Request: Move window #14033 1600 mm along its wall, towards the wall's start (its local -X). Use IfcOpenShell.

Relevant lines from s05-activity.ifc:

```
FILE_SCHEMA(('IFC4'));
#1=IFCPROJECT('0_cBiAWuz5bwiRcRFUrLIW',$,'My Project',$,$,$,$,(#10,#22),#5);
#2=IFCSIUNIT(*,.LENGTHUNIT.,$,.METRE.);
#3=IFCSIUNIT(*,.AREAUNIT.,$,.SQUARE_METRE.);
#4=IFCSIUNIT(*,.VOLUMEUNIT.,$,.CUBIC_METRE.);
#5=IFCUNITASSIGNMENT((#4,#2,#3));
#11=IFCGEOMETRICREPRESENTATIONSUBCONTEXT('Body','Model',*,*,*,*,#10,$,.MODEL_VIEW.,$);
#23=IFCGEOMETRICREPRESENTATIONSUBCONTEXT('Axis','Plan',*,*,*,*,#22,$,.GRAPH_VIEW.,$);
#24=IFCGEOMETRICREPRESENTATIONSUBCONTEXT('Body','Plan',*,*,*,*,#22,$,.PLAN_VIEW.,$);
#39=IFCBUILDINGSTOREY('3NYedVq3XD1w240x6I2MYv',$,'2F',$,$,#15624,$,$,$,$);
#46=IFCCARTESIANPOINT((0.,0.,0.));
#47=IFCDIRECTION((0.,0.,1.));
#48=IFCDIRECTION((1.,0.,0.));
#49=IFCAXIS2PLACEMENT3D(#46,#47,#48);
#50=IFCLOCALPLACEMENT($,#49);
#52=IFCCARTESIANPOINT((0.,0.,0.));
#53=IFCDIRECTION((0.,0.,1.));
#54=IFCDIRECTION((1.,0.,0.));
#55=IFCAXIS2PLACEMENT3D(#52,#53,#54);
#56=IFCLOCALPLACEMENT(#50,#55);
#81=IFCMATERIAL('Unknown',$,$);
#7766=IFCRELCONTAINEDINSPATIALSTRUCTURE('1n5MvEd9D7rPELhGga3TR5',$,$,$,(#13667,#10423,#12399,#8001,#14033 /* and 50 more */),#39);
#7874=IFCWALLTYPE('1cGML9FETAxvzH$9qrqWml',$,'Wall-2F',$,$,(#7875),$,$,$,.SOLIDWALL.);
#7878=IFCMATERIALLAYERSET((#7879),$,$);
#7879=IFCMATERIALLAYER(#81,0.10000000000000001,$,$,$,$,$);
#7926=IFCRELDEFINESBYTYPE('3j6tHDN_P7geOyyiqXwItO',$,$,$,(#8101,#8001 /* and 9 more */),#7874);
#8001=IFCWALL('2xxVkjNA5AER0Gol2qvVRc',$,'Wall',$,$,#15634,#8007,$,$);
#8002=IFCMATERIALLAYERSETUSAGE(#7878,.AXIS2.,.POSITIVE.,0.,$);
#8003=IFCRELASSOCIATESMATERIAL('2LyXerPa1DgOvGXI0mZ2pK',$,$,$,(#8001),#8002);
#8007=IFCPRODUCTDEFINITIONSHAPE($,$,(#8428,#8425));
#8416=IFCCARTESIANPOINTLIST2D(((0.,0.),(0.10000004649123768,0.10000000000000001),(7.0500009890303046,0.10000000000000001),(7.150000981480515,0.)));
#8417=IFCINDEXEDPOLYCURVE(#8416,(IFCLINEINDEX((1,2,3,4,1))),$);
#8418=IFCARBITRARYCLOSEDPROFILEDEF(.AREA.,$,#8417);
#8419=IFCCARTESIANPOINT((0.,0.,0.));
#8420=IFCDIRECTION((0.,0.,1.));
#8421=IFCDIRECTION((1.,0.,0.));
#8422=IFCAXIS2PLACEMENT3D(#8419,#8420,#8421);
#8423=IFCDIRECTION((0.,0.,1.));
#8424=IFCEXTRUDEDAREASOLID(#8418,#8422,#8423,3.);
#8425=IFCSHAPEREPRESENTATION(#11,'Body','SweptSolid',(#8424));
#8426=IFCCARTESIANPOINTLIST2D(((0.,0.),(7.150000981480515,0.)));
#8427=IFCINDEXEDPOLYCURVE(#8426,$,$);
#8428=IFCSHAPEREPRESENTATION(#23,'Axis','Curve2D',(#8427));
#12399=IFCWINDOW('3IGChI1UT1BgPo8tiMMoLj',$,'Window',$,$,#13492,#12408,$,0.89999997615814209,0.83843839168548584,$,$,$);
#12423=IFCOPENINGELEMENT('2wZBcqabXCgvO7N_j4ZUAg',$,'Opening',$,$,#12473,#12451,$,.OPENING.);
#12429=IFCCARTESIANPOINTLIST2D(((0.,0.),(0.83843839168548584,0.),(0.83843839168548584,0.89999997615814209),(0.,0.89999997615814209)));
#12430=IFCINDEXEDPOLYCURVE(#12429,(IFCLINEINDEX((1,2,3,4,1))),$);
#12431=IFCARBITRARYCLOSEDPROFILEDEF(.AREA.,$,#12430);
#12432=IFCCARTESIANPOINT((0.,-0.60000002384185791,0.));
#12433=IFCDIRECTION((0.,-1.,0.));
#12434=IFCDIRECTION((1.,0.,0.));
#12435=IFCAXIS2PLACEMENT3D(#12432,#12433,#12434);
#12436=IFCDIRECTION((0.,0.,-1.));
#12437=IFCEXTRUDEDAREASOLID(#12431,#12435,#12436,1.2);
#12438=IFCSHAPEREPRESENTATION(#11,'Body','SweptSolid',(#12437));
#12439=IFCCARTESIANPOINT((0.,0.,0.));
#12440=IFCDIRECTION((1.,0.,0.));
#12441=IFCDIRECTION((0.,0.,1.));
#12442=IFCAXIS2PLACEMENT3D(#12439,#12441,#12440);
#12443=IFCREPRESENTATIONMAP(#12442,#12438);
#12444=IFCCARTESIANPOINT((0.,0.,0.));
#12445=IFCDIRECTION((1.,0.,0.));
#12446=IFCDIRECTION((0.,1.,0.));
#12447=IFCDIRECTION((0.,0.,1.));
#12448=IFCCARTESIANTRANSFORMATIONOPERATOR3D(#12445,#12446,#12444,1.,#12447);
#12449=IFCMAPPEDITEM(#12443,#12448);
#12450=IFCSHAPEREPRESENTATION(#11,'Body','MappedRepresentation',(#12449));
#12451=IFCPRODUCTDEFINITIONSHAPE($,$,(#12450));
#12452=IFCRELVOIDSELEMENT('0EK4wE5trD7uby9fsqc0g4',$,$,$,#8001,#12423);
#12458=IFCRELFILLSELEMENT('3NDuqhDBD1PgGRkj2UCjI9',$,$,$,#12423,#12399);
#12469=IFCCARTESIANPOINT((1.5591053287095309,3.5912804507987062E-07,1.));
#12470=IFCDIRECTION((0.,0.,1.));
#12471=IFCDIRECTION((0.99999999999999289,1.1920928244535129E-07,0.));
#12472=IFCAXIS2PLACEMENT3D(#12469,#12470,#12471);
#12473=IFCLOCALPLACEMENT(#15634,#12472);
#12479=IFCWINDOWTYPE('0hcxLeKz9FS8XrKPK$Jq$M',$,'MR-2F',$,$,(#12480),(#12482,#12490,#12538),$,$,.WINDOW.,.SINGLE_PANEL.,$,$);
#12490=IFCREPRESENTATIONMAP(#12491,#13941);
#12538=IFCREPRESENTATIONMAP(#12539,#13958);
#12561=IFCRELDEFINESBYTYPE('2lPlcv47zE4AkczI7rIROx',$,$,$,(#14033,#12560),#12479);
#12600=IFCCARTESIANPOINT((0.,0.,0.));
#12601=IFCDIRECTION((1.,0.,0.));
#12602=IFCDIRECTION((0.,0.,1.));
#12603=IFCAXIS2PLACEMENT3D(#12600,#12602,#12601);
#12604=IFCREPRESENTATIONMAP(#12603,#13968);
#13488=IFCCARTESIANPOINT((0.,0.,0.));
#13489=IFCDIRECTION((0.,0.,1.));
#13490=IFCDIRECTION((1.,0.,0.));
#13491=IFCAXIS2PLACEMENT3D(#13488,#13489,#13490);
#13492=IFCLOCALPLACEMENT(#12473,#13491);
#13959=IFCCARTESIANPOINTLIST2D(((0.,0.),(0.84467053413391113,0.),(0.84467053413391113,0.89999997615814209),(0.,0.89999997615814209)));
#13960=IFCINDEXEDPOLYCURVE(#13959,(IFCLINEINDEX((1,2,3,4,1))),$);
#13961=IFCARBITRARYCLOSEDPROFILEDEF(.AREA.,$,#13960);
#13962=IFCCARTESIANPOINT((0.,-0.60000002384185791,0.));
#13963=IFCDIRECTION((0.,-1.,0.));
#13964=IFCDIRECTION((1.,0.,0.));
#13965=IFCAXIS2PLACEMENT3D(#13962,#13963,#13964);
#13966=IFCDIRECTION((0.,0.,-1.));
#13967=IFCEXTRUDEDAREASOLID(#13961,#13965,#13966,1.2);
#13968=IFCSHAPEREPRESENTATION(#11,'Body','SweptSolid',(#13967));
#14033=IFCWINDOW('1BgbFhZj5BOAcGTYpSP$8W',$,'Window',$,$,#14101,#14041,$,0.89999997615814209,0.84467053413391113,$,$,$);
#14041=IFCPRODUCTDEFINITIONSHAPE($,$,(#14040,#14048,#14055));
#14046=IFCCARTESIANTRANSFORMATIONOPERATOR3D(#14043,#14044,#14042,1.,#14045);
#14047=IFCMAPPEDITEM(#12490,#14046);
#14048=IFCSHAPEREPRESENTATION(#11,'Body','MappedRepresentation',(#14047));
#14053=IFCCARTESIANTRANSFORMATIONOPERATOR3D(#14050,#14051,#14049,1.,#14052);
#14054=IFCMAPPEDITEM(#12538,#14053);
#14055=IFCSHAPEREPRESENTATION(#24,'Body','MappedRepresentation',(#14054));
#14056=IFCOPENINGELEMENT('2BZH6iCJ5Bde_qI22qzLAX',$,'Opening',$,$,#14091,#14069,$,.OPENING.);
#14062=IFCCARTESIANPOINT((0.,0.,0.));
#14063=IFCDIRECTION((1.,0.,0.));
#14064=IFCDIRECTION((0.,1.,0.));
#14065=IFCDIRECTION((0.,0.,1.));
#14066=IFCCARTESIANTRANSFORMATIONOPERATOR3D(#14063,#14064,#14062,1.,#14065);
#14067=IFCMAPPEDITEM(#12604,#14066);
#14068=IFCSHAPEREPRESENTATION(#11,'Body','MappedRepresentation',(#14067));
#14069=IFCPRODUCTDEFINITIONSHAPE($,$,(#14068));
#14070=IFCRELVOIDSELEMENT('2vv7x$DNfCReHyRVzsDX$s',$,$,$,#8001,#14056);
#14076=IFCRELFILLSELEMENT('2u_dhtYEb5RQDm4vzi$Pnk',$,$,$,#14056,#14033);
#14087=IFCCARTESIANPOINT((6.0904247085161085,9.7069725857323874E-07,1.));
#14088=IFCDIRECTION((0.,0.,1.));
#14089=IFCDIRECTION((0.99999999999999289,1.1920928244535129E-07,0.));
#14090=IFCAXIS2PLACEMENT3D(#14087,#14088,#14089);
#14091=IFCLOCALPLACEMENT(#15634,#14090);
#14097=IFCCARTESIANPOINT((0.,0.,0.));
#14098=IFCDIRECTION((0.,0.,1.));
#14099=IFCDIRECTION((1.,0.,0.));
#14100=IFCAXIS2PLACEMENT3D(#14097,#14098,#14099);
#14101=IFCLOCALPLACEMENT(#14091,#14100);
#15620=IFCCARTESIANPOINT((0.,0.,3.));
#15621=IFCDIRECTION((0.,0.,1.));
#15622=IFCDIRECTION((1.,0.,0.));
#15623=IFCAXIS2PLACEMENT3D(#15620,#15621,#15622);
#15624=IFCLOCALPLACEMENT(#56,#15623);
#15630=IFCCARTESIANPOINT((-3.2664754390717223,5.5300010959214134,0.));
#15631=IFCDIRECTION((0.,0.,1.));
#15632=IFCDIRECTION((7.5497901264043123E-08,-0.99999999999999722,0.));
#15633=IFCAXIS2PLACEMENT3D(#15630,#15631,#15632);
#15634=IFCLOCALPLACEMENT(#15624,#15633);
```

```python
import ifcopenshell
import ifcopenshell.api.geometry
import ifcopenshell.util.placement
import ifcopenshell.util.unit

model = ifcopenshell.open("s05-activity.ifc")
unit_scale = ifcopenshell.util.unit.calculate_unit_scale(model)

window = model.by_guid("1BgbFhZj5BOAcGTYpSP$8W")
opening = window.FillsVoids[0].RelatingOpeningElement
wall = opening.VoidsElements[0].RelatingBuildingElement

wall_matrix = ifcopenshell.util.placement.get_local_placement(wall.ObjectPlacement)
shift = wall_matrix[:3, 0] * -1.6 / unit_scale
before = ifcopenshell.util.placement.get_local_placement(window.ObjectPlacement)[:3, 3].copy()

# The window is placed relative to its opening, so it follows when the opening moves.
matrix = ifcopenshell.util.placement.get_local_placement(opening.ObjectPlacement)
matrix[:3, 3] += shift
ifcopenshell.api.geometry.edit_object_placement(
    model, product=opening, matrix=matrix, is_si=False, should_transform_children=True
)

after = ifcopenshell.util.placement.get_local_placement(window.ObjectPlacement)[:3, 3]
print("window moved by", (after - before).round(3) + 0.0)

model.write("s05-activity_updated.ifc")
```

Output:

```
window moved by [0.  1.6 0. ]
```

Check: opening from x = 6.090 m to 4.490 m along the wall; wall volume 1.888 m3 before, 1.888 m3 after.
